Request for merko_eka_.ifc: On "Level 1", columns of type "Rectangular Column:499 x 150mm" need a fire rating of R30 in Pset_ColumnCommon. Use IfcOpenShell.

First a look at what the model holds.

```python
import ifcopenshell
import ifcopenshell.util.element

model = ifcopenshell.open("merko_eka_.ifc")
print(model.schema)
storey = next(s for s in model.by_type("IfcBuildingStorey") if s.Name == "Level 1")
columns = [e for e in ifcopenshell.util.element.get_decomposition(storey) if e.is_a("IfcColumn")]
seen = {}
for e in columns:
    element_type = ifcopenshell.util.element.get_type(e)
    key = (element_type.Name if element_type != e and element_type else None, ifcopenshell.util.element.get_pset(e, "Pset_ColumnCommon", "FireRating"))
    seen[key] = seen.get(key, 0) + 1
for (name, value), count in sorted(seen.items(), key=str):
    print(count, "x", name, "|", value)
```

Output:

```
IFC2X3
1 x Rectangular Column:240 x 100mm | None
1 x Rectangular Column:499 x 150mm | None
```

```python
import ifcopenshell
import ifcopenshell.api.pset
import ifcopenshell.util.element

model = ifcopenshell.open("merko_eka_.ifc")

storey = next(s for s in model.by_type("IfcBuildingStorey") if s.Name == "Level 1")
columns = [e for e in ifcopenshell.util.element.get_decomposition(storey) if e.is_a("IfcColumn")]

count = 0
for e in columns:
    element_type = ifcopenshell.util.element.get_type(e)
    if element_type in (None, e) or element_type.Name != "Rectangular Column:499 x 150mm":
        continue
    # add_pset returns the element's existing set when there is one.
    pset = ifcopenshell.api.pset.add_pset(model, product=e, name="Pset_ColumnCommon")
    ifcopenshell.api.pset.edit_pset(model, pset=pset, properties={"FireRating": "R30"})
    count += 1

print(count, "columns updated")

model.write("merko_eka__edited.ifc")
```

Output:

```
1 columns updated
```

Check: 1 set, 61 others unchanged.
